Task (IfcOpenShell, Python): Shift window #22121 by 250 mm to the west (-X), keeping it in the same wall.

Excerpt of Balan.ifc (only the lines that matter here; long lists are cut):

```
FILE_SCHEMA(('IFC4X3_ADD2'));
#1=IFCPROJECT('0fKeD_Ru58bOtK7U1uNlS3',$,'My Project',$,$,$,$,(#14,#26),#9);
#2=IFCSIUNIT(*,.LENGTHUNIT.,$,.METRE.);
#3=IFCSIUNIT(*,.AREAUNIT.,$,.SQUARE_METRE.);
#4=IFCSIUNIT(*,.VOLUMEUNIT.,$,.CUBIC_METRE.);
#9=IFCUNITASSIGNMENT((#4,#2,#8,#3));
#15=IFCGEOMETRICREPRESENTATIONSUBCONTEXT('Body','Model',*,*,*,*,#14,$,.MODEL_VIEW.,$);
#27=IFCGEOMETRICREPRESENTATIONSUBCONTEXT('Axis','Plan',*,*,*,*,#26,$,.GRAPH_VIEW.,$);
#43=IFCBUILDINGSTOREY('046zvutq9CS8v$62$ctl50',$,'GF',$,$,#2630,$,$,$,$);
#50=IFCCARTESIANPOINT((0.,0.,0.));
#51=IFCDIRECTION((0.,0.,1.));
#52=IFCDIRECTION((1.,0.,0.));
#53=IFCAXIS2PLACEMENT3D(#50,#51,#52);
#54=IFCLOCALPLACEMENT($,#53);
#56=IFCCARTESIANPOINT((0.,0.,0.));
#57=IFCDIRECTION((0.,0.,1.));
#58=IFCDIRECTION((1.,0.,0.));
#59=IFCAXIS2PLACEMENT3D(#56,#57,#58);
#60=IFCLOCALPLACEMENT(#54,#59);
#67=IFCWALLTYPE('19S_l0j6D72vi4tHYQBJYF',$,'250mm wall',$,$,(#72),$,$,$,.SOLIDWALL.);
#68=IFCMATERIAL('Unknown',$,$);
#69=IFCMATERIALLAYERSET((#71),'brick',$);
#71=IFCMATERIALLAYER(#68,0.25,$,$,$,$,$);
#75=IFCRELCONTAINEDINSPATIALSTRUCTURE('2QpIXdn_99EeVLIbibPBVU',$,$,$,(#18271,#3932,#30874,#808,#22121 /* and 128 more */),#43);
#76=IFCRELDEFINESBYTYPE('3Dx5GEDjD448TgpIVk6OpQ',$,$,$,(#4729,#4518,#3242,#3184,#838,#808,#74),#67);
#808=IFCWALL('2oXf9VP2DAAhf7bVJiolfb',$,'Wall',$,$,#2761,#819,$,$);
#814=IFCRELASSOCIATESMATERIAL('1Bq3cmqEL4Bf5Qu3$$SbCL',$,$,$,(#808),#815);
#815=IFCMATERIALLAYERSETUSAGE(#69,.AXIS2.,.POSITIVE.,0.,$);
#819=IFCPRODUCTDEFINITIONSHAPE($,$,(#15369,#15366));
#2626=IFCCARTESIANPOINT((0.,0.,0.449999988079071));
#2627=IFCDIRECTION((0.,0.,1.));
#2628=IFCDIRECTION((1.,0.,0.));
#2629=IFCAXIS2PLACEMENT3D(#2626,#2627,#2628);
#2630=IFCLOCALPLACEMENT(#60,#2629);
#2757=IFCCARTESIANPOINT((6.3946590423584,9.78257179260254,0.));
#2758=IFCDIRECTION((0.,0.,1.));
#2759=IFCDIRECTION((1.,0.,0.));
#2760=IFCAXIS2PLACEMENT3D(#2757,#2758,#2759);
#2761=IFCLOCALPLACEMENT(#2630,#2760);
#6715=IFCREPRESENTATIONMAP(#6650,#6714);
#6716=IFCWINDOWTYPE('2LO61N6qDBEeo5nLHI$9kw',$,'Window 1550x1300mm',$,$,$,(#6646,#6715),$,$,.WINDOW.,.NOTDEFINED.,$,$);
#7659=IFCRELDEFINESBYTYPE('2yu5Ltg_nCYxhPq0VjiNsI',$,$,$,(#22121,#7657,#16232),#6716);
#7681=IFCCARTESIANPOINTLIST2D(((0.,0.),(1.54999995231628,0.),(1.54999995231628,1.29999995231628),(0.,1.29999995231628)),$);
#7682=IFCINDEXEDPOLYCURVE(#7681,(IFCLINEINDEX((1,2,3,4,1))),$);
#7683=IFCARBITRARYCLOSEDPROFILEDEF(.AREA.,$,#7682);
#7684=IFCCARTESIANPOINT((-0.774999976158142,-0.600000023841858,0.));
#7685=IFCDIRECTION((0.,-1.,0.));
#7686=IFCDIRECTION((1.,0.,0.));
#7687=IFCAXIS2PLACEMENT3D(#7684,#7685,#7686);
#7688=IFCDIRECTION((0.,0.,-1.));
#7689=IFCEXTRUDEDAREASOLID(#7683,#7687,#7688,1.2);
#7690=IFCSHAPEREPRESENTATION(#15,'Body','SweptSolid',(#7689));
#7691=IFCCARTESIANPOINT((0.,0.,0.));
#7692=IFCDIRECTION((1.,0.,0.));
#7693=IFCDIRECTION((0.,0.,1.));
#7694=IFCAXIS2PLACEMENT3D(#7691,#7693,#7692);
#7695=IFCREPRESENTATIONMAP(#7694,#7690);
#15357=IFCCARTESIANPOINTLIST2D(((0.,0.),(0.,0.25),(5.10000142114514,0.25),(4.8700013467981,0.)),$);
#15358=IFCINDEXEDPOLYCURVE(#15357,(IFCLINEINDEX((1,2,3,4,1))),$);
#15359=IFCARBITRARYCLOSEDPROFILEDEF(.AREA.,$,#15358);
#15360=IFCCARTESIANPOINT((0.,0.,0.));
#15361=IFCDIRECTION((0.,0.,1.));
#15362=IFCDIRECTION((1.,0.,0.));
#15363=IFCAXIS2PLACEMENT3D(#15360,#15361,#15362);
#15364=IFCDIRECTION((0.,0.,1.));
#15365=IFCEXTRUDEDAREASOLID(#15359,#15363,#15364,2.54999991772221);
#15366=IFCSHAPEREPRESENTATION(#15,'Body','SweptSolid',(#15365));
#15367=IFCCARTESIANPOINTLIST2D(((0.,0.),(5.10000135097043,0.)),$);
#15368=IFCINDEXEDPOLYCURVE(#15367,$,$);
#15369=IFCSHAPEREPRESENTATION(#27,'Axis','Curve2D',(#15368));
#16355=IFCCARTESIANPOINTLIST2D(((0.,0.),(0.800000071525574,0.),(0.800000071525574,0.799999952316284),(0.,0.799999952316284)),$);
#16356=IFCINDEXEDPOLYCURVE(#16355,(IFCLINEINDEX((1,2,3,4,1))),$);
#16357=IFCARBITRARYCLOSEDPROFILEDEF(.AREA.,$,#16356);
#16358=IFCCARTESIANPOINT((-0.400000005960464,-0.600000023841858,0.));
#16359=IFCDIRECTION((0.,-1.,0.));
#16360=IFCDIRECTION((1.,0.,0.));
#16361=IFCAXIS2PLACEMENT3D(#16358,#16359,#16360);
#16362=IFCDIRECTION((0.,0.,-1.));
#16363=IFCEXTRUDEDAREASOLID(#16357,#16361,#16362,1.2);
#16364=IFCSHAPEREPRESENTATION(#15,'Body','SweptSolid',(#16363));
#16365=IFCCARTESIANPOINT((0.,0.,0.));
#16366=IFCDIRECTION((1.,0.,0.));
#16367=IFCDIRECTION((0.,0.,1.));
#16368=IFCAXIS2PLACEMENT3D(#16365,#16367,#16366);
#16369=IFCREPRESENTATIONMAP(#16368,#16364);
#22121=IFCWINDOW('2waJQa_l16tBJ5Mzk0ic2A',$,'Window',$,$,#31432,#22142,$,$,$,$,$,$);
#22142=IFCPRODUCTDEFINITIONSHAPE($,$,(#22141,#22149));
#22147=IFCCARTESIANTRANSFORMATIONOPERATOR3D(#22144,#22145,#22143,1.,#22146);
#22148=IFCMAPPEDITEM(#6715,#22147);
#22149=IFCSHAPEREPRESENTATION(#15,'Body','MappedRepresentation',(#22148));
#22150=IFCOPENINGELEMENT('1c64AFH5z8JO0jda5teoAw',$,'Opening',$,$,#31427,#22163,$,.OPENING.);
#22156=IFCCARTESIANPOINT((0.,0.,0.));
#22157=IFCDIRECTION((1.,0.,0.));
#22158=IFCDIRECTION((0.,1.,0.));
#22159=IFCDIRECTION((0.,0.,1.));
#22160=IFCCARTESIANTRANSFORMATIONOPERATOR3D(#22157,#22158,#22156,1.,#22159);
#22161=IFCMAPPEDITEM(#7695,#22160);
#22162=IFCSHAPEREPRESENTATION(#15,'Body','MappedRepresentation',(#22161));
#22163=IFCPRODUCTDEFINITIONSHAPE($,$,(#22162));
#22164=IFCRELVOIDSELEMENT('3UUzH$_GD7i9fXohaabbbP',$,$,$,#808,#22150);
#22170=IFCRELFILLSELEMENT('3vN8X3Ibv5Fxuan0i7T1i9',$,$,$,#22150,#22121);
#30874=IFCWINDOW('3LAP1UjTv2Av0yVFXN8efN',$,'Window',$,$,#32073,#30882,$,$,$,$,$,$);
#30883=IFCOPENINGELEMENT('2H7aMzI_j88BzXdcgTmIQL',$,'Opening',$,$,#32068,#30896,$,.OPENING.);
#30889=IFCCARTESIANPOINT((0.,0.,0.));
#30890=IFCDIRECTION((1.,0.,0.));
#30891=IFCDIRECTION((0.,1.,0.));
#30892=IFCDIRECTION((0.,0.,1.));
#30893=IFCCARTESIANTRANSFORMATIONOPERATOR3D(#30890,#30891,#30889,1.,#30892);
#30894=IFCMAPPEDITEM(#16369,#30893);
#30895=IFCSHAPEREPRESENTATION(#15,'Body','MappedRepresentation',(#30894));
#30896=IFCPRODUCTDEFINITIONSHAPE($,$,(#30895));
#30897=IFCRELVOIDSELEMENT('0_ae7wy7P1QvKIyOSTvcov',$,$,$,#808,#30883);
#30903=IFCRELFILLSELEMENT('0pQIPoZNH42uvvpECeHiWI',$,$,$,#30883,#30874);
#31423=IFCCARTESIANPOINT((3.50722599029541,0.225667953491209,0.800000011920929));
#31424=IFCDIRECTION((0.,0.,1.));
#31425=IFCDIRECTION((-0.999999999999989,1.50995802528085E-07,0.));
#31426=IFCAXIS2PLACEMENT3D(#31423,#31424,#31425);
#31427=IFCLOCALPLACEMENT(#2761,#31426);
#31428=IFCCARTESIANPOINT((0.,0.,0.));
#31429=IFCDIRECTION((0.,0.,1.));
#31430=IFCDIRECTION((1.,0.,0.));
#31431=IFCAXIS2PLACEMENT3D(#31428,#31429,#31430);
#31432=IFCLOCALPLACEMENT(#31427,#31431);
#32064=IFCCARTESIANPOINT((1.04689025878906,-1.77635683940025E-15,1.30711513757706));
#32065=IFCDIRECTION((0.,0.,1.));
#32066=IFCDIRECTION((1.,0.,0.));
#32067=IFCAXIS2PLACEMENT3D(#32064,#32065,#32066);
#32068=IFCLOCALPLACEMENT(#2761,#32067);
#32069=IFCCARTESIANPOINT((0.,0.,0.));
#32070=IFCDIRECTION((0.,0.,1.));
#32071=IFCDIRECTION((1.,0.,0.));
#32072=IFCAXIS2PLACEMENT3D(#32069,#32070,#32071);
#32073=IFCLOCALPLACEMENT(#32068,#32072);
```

```python
import ifcopenshell
import ifcopenshell.api.geometry
import ifcopenshell.util.placement

model = ifcopenshell.open("Balan.ifc")

window = model.by_guid("2waJQa_l16tBJ5Mzk0ic2A")
opening = window.FillsVoids[0].RelatingOpeningElement
wall = opening.VoidsElements[0].RelatingBuildingElement

wall_matrix = ifcopenshell.util.placement.get_local_placement(wall.ObjectPlacement)
shift = wall_matrix[:3, 0] * -0.25
before = ifcopenshell.util.placement.get_local_placement(window.ObjectPlacement)[:3, 3].copy()

# The window is placed relative to its opening, so it follows when the opening moves.
matrix = ifcopenshell.util.placement.get_local_placement(opening.ObjectPlacement)
matrix[:3, 3] += shift
ifcopenshell.api.geometry.edit_object_placement(
    model, product=opening, matrix=matrix, is_si=False, should_transform_children=True
)

after = ifcopenshell.util.placement.get_local_placement(window.ObjectPlacement)[:3, 3]
print("window moved by", (after - before).round(3) + 0.0)

model.write("Balan-out.ifc")
```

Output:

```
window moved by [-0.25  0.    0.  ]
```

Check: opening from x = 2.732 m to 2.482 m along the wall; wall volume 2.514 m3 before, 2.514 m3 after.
